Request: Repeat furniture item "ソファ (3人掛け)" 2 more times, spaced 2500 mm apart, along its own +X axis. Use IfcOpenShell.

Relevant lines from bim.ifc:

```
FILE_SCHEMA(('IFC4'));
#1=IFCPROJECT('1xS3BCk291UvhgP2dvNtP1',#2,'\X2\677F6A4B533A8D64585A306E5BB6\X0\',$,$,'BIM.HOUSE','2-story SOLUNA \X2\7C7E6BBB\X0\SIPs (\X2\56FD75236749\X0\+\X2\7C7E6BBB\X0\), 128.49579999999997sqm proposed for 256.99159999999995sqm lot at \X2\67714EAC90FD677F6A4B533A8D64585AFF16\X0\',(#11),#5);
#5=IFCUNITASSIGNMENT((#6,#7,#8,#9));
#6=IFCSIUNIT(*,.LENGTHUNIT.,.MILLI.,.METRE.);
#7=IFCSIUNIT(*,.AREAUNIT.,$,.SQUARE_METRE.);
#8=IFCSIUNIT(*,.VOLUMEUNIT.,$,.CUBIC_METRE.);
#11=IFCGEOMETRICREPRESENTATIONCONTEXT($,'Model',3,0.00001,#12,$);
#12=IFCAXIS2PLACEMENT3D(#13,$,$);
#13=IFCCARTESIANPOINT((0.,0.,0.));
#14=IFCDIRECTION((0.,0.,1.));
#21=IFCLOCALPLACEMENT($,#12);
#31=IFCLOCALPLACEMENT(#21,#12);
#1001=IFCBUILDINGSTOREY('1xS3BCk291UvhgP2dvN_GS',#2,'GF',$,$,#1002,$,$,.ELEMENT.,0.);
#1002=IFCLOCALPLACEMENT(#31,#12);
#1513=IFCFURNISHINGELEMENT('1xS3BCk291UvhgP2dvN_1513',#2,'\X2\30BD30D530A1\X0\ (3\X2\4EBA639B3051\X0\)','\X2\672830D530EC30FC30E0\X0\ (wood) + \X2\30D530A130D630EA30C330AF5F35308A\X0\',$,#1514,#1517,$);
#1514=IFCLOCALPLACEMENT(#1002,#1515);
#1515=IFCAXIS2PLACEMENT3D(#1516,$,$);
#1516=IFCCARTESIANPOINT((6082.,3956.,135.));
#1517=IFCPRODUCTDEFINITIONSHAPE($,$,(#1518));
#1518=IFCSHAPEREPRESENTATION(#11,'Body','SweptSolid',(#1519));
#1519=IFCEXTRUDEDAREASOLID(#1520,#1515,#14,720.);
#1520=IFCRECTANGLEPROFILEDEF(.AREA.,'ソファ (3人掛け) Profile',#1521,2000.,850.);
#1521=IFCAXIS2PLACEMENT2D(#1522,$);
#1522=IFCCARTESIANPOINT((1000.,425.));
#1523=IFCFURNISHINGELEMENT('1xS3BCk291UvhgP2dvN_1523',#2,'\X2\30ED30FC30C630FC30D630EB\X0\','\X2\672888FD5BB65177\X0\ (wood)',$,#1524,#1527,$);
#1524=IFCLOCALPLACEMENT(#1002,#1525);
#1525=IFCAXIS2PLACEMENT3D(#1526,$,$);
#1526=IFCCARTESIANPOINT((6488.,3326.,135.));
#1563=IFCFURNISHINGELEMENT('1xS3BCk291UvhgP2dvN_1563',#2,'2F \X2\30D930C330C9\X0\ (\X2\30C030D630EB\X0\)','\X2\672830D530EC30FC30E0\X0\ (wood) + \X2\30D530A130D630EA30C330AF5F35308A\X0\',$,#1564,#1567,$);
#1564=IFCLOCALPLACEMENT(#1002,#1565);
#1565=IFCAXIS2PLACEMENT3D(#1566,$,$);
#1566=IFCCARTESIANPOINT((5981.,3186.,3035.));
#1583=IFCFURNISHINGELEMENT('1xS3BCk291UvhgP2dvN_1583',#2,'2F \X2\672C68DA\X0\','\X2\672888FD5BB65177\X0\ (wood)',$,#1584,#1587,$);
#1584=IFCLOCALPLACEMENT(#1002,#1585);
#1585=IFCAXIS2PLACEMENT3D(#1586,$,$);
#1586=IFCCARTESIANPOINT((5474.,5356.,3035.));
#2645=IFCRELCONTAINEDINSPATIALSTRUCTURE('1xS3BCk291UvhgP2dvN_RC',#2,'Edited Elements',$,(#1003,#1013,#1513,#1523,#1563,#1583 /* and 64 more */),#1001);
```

```python
import ifcopenshell
import ifcopenshell.api.geometry
import ifcopenshell.api.root
import ifcopenshell.util.element
import ifcopenshell.util.placement

model = ifcopenshell.open("bim.ifc")


def reuse_history(source, copy):
    """copy_class also copies each property set's owner history, people and application; keep the originals."""
    for rel in copy.IsDefinedBy:
        if rel.is_a("IfcRelDefinesByProperties") and (history := rel.RelatingPropertyDefinition.OwnerHistory):
            rel.RelatingPropertyDefinition.OwnerHistory = source.OwnerHistory
            ifcopenshell.util.element.remove_deep2(model, history)


source = model.by_guid("1xS3BCk291UvhgP2dvN_1513")
base = ifcopenshell.util.placement.get_local_placement(source.ObjectPlacement)
step = base[:3, 0] * 2500.0

for i in range(1, 3):
    copy = ifcopenshell.api.root.copy_class(model, product=source)
    copy.Representation = ifcopenshell.util.element.copy_deep(
        model, source.Representation, exclude=["IfcGeometricRepresentationContext", "IfcRepresentationMap"]
    )
    reuse_history(source, copy)
    matrix = base.copy()
    matrix[:3, 3] += i * step
    print("added at", matrix[:3, 3].round(3) + 0.0)
    ifcopenshell.api.geometry.edit_object_placement(model, product=copy, matrix=matrix, is_si=False)

model.write("bim_v2.ifc")
```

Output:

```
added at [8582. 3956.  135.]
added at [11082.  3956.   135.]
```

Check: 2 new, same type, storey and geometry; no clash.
